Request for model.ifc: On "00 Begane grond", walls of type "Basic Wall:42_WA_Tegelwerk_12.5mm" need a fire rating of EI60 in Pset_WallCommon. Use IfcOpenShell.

First a look at what the model holds.

```python
import ifcopenshell
import ifcopenshell.util.element

model = ifcopenshell.open("model.ifc")
print(model.schema)
storey = next(s for s in model.by_type("IfcBuildingStorey") if s.Name == "00 Begane grond")
walls = [e for e in ifcopenshell.util.element.get_decomposition(storey) if e.is_a("IfcWall")]
seen = {}
for e in walls:
    element_type = ifcopenshell.util.element.get_type(e)
    key = (element_type.Name if element_type != e and element_type else None, ifcopenshell.util.element.get_pset(e, "Pset_WallCommon", "FireRating"))
    seen[key] = seen.get(key, 0) + 1
for (name, value), count in sorted(seen.items(), key=str):
    print(count, "x", name, "|", value)
```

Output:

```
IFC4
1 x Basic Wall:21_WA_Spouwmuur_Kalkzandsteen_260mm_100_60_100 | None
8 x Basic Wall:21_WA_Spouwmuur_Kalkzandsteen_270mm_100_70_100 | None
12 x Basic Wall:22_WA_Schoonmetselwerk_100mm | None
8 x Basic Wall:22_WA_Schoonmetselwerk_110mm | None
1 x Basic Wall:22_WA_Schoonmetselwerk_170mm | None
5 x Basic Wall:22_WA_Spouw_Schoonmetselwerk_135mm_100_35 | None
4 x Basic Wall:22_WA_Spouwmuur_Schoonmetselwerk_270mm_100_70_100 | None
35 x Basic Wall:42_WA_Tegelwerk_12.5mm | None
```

```python
import ifcopenshell
import ifcopenshell.api.pset
import ifcopenshell.util.element

model = ifcopenshell.open("model.ifc")

storey = next(s for s in model.by_type("IfcBuildingStorey") if s.Name == "00 Begane grond")
walls = [e for e in ifcopenshell.util.element.get_decomposition(storey) if e.is_a("IfcWall")]

count = 0
for e in walls:
    element_type = ifcopenshell.util.element.get_type(e)
    if element_type in (None, e) or element_type.Name != "Basic Wall:42_WA_Tegelwerk_12.5mm":
        continue
    # add_pset returns the element's existing set when there is one.
    pset = ifcopenshell.api.pset.add_pset(model, product=e, name="Pset_WallCommon")
    ifcopenshell.api.pset.edit_pset(model, pset=pset, properties={"FireRating": "EI60"})
    count += 1

print(count, "walls updated")

model.write("model_rev.ifc")
```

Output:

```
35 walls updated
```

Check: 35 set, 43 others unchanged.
